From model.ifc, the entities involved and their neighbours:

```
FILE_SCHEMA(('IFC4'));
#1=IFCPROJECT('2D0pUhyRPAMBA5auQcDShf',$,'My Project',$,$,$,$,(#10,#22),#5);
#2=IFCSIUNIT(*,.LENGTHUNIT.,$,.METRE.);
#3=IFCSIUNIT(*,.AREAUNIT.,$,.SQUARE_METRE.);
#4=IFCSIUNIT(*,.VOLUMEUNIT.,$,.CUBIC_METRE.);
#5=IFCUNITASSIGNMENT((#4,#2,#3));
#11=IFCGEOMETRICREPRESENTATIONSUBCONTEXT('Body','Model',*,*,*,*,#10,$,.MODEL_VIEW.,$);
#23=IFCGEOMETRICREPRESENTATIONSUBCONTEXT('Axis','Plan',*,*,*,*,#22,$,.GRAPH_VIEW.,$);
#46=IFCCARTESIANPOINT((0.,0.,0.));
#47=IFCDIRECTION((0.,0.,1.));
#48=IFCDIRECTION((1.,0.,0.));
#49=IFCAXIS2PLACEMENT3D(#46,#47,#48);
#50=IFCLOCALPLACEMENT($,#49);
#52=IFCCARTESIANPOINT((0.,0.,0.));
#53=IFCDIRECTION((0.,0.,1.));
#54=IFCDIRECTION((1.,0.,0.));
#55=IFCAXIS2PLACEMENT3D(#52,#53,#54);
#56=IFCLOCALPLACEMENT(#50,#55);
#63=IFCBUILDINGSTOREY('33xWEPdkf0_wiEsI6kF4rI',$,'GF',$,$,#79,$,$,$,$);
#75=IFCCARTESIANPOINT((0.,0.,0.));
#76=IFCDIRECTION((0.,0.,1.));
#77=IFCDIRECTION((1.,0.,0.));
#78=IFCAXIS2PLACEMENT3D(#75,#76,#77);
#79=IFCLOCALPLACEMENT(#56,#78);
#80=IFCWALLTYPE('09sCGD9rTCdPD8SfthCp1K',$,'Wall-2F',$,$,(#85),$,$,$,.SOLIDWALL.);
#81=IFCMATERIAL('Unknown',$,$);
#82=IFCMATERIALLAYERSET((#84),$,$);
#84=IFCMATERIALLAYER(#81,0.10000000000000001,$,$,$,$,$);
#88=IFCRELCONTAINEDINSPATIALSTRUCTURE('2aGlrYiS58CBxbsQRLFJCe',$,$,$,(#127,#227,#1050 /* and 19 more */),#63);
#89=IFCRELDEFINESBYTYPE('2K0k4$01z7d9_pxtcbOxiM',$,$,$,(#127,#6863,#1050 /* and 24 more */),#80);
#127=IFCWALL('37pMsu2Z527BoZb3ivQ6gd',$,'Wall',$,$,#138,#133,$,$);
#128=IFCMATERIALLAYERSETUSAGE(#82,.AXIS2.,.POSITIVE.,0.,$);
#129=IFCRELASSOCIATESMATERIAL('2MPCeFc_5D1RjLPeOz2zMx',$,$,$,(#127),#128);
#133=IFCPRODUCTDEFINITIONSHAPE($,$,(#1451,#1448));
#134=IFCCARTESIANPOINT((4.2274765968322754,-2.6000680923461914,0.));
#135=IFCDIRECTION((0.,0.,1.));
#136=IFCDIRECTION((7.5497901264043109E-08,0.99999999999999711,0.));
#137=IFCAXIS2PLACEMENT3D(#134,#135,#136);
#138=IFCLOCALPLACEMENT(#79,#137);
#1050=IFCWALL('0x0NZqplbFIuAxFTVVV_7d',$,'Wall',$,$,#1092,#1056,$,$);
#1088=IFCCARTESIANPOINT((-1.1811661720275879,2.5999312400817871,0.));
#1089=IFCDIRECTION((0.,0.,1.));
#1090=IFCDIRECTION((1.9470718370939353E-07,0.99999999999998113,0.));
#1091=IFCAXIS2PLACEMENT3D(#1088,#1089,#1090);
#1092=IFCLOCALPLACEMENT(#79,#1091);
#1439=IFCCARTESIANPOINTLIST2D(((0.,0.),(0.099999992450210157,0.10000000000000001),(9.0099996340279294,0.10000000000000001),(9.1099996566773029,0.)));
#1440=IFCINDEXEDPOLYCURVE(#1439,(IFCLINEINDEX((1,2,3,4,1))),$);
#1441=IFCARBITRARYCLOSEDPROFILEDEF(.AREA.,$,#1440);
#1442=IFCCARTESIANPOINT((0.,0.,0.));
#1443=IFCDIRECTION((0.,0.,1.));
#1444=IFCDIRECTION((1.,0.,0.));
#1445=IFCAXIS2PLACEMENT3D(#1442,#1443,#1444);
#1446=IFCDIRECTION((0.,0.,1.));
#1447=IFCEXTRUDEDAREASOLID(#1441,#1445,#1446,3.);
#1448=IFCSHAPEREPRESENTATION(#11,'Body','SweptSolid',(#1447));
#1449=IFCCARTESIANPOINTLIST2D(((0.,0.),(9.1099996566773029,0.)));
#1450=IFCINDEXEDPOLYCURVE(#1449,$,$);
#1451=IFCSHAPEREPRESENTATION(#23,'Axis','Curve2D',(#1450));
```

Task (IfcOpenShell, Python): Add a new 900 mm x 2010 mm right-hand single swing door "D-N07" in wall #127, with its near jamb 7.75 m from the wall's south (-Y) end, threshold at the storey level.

```python
import numpy as np
import ifcopenshell
import ifcopenshell.api.feature
import ifcopenshell.api.geometry
import ifcopenshell.api.root
import ifcopenshell.api.spatial
import ifcopenshell.geom
import ifcopenshell.util.element
import ifcopenshell.util.placement
import ifcopenshell.util.representation
import ifcopenshell.util.shape
import ifcopenshell.util.unit

model = ifcopenshell.open("model.ifc")
unit_scale = ifcopenshell.util.unit.calculate_unit_scale(model)
settings = ifcopenshell.geom.settings()


def volume(element):
    """Net volume in cubic metres, openings subtracted."""
    shape = ifcopenshell.geom.create_shape(settings, element)
    return ifcopenshell.util.shape.get_volume(shape.geometry)


wall = model.by_guid("37pMsu2Z527BoZb3ivQ6gd")
storey = ifcopenshell.util.element.get_container(wall, ifc_class="IfcBuildingStorey")
context = ifcopenshell.util.representation.get_context(model, "Model", "Body", "MODEL_VIEW")
before = volume(wall)

width, height, from_end, sill = 0.9, 2.01, 7.75, 0.0  # metres

# The wall runs along its own X axis, and the end named is its -X end.
wall_shape = ifcopenshell.geom.create_shape(settings, wall)
x, y, z = ifcopenshell.util.shape.get_vertices(wall_shape.geometry).T
start = x.min() + from_end
face, thickness = float(y.min()), float(y.max() - y.min())
wall_matrix = ifcopenshell.util.placement.get_local_placement(wall.ObjectPlacement)
level = ifcopenshell.util.placement.get_local_placement(storey.ObjectPlacement)[2, 3]


def in_wall(x, y):
    """Placement at x, y metres in the wall's axes, at sill height."""
    matrix = wall_matrix.copy()
    matrix[:, 3] = wall_matrix @ np.array([x / unit_scale, y / unit_scale, 0.0, 1.0])
    matrix[2, 3] = level + sill / unit_scale
    return matrix


# Opening: a box that overshoots both wall faces by 50 mm.
opening = ifcopenshell.api.root.create_entity(model, ifc_class="IfcOpeningElement", predefined_type="OPENING")
box = ifcopenshell.api.geometry.add_wall_representation(
    model, context=context, length=width, height=height, thickness=thickness + 0.1
)
ifcopenshell.api.geometry.assign_representation(model, product=opening, representation=box)
ifcopenshell.api.geometry.edit_object_placement(model, product=opening, matrix=in_wall(start, face - 0.05), is_si=False)
ifcopenshell.api.feature.add_feature(model, feature=opening, element=wall)

door = ifcopenshell.api.root.create_entity(model, ifc_class="IfcDoor", name="D-N07", predefined_type="DOOR")
door.OverallWidth, door.OverallHeight = width / unit_scale, height / unit_scale
door.OperationType = "SINGLE_SWING_RIGHT"
body = ifcopenshell.api.geometry.add_door_representation(
    model,
    context=context,
    overall_width=door.OverallWidth,
    overall_height=door.OverallHeight,
    operation_type="SINGLE_SWING_RIGHT",
    lining_properties={"LiningDepth": thickness / unit_scale, "ThresholdDepth": thickness / unit_scale},
)
ifcopenshell.api.geometry.assign_representation(model, product=door, representation=body)
ifcopenshell.api.spatial.assign_container(model, products=[door], relating_structure=storey)
ifcopenshell.api.feature.add_filling(model, opening=opening, element=door)

# The lining spans the wall, so the door starts at the wall face.
ifcopenshell.api.geometry.edit_object_placement(model, product=door, matrix=in_wall(start, face), is_si=False)

after = volume(wall)

print(f"wall volume {before:.3f} -> {after:.3f} m3")

model.write("model-out.ifc")
```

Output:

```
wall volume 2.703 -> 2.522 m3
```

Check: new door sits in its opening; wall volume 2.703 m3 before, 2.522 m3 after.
